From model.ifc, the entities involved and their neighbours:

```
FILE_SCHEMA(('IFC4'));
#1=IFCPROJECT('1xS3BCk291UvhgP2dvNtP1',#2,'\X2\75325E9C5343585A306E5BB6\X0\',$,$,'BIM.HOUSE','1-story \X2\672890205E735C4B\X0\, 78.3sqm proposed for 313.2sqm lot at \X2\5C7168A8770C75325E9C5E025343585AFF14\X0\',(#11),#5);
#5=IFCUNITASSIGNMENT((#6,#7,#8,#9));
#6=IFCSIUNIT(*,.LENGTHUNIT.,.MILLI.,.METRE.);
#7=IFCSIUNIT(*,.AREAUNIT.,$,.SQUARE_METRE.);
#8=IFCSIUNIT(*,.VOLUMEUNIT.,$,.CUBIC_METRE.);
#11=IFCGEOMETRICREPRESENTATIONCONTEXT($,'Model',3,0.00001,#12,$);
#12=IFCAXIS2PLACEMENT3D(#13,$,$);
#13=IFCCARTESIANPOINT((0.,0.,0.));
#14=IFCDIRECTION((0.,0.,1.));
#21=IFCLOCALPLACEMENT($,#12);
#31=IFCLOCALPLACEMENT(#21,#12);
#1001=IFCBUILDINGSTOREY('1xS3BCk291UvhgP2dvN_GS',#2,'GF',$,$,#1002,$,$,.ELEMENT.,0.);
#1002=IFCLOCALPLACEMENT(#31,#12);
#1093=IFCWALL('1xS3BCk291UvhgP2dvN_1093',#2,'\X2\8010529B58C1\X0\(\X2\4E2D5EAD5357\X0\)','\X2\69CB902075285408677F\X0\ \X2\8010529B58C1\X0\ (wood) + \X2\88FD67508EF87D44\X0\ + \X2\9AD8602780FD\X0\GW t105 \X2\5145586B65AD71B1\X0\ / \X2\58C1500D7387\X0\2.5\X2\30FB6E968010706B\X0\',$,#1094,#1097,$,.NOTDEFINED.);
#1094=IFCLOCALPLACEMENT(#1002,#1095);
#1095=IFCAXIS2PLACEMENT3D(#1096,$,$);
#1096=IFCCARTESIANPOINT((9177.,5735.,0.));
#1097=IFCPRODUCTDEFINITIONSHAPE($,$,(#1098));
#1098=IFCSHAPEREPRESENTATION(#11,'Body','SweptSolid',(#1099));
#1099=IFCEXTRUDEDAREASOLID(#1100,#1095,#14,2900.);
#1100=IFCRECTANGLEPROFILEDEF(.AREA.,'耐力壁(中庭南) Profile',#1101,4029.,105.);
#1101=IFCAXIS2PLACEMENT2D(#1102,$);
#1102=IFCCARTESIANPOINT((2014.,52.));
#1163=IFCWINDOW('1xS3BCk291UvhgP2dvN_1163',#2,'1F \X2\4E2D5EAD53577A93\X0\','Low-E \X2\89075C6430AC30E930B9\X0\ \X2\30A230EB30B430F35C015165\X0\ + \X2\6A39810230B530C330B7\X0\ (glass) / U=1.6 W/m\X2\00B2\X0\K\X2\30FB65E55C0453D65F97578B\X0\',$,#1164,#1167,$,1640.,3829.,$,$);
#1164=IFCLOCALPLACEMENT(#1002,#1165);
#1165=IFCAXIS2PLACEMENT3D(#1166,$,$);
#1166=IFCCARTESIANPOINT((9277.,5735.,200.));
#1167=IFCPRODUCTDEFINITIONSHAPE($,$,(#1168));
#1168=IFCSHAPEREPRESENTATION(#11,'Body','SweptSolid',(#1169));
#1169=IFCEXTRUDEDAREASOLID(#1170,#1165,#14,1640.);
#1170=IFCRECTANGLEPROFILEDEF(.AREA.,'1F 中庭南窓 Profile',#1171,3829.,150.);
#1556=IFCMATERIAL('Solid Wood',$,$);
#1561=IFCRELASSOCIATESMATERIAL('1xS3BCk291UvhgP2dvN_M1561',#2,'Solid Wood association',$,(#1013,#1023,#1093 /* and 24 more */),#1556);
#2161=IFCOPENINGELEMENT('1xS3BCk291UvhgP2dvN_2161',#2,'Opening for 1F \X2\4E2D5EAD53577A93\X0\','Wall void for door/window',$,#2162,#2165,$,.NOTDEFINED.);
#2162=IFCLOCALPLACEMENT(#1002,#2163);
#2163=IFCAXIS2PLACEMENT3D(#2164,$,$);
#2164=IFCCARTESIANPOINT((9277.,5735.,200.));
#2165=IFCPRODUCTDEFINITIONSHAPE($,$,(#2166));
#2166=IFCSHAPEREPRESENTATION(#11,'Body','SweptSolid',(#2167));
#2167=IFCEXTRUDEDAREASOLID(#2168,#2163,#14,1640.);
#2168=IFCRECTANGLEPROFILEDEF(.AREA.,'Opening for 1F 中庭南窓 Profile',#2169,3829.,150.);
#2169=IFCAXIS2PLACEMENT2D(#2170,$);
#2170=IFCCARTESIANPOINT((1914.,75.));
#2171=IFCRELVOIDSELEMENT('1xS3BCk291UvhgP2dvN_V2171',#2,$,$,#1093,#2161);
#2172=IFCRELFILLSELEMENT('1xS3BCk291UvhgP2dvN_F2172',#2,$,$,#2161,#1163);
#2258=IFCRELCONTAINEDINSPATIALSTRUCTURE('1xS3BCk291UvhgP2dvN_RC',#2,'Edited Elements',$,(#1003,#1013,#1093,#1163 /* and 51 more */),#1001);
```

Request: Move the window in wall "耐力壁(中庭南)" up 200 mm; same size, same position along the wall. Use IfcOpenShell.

```python
import numpy as np
import ifcopenshell
import ifcopenshell.api.geometry
import ifcopenshell.util.placement
import ifcopenshell.util.unit

model = ifcopenshell.open("model.ifc")
unit_scale = ifcopenshell.util.unit.calculate_unit_scale(model)

window = model.by_id(1163)
opening = window.FillsVoids[0].RelatingOpeningElement
dz = 200.0

shift = np.array([0.0, 0.0, dz])
# The window is not placed relative to its opening, so move both.
for product in (opening, window):
    matrix = ifcopenshell.util.placement.get_local_placement(product.ObjectPlacement)
    matrix[:3, 3] += shift
    ifcopenshell.api.geometry.edit_object_placement(model, product=product, matrix=matrix, is_si=False)

print(f"moved by {dz * unit_scale:+.3f} m")

model.write("model-out.ifc")
```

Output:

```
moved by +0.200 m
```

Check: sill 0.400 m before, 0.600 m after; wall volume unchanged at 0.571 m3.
